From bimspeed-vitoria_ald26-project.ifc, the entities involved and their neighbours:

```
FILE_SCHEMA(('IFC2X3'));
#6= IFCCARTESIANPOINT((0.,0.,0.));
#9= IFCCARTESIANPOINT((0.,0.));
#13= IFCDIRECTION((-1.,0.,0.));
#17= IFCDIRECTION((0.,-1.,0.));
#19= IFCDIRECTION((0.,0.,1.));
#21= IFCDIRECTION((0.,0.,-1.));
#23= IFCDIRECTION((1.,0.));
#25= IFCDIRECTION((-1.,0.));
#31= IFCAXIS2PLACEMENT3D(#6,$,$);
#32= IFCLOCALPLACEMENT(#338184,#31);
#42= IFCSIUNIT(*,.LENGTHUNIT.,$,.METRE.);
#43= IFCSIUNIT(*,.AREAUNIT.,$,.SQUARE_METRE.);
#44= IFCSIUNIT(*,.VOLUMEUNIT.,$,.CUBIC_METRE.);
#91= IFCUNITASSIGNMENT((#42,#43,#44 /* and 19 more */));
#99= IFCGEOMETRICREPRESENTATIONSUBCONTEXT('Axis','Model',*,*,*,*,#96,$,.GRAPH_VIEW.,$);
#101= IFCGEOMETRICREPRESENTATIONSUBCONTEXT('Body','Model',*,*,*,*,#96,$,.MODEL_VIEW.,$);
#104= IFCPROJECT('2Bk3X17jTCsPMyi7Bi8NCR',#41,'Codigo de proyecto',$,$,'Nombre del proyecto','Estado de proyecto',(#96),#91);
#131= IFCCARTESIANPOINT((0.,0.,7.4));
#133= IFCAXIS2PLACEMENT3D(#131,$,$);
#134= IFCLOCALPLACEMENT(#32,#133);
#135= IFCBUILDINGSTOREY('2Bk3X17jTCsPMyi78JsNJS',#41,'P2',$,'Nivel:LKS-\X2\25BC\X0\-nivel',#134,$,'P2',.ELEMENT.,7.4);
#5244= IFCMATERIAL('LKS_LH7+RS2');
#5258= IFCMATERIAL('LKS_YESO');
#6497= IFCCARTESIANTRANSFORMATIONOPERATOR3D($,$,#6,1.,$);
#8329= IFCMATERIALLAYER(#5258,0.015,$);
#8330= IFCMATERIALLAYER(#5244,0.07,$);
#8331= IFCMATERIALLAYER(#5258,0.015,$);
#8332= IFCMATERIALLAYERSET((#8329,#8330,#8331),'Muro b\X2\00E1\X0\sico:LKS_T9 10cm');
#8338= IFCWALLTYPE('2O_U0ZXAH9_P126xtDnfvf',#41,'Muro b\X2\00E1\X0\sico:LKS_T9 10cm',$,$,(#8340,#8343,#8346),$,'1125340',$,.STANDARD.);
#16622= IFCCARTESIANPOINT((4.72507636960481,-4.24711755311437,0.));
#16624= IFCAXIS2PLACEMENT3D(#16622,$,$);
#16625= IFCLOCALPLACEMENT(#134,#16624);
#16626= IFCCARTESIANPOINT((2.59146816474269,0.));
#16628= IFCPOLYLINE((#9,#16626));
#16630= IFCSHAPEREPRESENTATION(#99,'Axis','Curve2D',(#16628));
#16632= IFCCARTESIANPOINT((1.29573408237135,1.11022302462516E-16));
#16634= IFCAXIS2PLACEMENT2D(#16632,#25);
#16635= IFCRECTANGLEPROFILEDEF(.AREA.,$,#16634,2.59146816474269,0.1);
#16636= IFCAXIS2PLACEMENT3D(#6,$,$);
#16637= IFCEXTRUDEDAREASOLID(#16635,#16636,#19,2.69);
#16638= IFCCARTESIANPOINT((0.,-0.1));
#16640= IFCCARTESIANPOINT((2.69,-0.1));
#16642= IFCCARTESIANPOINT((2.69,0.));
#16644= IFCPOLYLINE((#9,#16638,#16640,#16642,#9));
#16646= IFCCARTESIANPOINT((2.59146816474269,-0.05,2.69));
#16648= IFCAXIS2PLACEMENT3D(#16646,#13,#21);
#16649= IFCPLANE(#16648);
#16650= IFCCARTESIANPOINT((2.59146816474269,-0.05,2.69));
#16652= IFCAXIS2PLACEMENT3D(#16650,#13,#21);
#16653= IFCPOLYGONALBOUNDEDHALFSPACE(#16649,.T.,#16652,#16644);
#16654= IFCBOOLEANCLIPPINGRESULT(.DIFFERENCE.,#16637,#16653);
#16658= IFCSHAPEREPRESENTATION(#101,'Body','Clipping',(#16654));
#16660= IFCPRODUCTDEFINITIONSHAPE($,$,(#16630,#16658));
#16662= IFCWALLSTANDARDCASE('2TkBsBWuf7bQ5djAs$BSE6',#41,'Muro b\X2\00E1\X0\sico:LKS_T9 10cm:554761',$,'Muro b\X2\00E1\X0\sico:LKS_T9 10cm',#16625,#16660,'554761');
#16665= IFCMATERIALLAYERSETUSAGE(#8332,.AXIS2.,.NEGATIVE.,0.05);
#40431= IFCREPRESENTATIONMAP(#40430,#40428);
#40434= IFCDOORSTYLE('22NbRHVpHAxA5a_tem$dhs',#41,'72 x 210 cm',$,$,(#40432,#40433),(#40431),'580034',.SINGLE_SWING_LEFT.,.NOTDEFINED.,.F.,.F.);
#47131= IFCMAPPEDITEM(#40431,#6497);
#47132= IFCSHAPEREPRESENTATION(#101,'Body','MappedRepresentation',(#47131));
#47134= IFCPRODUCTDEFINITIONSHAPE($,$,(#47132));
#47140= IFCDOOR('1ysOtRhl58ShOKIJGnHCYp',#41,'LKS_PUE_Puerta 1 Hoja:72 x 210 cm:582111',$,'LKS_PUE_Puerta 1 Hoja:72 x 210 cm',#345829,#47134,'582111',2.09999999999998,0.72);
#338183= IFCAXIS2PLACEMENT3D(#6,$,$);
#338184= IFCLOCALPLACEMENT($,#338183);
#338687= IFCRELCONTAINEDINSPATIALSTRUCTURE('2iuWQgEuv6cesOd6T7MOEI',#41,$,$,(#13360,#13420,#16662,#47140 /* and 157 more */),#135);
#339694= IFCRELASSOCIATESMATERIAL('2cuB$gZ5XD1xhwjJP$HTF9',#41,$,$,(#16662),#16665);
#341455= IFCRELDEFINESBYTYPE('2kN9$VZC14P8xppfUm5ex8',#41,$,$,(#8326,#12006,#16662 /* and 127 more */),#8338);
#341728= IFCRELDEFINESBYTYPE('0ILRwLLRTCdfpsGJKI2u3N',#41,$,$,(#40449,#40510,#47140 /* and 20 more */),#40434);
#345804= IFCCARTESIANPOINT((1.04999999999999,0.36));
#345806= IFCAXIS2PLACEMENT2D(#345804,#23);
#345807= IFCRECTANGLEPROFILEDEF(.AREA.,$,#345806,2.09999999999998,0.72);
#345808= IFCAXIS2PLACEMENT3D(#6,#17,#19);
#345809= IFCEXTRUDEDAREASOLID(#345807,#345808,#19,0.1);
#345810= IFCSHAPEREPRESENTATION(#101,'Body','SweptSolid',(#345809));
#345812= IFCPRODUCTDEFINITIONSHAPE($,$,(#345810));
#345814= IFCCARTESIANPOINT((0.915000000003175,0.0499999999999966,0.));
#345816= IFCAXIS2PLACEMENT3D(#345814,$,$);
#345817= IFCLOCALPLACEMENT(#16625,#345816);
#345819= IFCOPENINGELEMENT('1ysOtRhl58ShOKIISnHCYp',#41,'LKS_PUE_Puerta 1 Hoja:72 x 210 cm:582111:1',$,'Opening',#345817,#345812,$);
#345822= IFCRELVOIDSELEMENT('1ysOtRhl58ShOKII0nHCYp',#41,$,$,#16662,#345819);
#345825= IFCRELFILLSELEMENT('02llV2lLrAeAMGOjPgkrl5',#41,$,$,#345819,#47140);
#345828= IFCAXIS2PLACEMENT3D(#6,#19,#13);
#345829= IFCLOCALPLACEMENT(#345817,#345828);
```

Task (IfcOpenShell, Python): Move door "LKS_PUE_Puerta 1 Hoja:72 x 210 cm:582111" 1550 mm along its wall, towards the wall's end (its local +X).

```python
import ifcopenshell
import ifcopenshell.api.geometry
import ifcopenshell.util.placement
import ifcopenshell.util.unit

model = ifcopenshell.open("bimspeed-vitoria_ald26-project.ifc")
unit_scale = ifcopenshell.util.unit.calculate_unit_scale(model)

door = model.by_guid("1ysOtRhl58ShOKIJGnHCYp")
opening = door.FillsVoids[0].RelatingOpeningElement
wall = opening.VoidsElements[0].RelatingBuildingElement

wall_matrix = ifcopenshell.util.placement.get_local_placement(wall.ObjectPlacement)
shift = wall_matrix[:3, 0] * 1.55 / unit_scale
before = ifcopenshell.util.placement.get_local_placement(door.ObjectPlacement)[:3, 3].copy()

# The door is placed relative to its opening, so it follows when the opening moves.
matrix = ifcopenshell.util.placement.get_local_placement(opening.ObjectPlacement)
matrix[:3, 3] += shift
ifcopenshell.api.geometry.edit_object_placement(
    model, product=opening, matrix=matrix, is_si=False, should_transform_children=True
)

after = ifcopenshell.util.placement.get_local_placement(door.ObjectPlacement)[:3, 3]
print("door moved by", (after - before).round(3) + 0.0)

model.write("bimspeed-vitoria_ald26-project_edited.ifc")
```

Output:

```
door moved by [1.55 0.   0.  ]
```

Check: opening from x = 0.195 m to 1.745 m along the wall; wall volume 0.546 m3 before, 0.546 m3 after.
